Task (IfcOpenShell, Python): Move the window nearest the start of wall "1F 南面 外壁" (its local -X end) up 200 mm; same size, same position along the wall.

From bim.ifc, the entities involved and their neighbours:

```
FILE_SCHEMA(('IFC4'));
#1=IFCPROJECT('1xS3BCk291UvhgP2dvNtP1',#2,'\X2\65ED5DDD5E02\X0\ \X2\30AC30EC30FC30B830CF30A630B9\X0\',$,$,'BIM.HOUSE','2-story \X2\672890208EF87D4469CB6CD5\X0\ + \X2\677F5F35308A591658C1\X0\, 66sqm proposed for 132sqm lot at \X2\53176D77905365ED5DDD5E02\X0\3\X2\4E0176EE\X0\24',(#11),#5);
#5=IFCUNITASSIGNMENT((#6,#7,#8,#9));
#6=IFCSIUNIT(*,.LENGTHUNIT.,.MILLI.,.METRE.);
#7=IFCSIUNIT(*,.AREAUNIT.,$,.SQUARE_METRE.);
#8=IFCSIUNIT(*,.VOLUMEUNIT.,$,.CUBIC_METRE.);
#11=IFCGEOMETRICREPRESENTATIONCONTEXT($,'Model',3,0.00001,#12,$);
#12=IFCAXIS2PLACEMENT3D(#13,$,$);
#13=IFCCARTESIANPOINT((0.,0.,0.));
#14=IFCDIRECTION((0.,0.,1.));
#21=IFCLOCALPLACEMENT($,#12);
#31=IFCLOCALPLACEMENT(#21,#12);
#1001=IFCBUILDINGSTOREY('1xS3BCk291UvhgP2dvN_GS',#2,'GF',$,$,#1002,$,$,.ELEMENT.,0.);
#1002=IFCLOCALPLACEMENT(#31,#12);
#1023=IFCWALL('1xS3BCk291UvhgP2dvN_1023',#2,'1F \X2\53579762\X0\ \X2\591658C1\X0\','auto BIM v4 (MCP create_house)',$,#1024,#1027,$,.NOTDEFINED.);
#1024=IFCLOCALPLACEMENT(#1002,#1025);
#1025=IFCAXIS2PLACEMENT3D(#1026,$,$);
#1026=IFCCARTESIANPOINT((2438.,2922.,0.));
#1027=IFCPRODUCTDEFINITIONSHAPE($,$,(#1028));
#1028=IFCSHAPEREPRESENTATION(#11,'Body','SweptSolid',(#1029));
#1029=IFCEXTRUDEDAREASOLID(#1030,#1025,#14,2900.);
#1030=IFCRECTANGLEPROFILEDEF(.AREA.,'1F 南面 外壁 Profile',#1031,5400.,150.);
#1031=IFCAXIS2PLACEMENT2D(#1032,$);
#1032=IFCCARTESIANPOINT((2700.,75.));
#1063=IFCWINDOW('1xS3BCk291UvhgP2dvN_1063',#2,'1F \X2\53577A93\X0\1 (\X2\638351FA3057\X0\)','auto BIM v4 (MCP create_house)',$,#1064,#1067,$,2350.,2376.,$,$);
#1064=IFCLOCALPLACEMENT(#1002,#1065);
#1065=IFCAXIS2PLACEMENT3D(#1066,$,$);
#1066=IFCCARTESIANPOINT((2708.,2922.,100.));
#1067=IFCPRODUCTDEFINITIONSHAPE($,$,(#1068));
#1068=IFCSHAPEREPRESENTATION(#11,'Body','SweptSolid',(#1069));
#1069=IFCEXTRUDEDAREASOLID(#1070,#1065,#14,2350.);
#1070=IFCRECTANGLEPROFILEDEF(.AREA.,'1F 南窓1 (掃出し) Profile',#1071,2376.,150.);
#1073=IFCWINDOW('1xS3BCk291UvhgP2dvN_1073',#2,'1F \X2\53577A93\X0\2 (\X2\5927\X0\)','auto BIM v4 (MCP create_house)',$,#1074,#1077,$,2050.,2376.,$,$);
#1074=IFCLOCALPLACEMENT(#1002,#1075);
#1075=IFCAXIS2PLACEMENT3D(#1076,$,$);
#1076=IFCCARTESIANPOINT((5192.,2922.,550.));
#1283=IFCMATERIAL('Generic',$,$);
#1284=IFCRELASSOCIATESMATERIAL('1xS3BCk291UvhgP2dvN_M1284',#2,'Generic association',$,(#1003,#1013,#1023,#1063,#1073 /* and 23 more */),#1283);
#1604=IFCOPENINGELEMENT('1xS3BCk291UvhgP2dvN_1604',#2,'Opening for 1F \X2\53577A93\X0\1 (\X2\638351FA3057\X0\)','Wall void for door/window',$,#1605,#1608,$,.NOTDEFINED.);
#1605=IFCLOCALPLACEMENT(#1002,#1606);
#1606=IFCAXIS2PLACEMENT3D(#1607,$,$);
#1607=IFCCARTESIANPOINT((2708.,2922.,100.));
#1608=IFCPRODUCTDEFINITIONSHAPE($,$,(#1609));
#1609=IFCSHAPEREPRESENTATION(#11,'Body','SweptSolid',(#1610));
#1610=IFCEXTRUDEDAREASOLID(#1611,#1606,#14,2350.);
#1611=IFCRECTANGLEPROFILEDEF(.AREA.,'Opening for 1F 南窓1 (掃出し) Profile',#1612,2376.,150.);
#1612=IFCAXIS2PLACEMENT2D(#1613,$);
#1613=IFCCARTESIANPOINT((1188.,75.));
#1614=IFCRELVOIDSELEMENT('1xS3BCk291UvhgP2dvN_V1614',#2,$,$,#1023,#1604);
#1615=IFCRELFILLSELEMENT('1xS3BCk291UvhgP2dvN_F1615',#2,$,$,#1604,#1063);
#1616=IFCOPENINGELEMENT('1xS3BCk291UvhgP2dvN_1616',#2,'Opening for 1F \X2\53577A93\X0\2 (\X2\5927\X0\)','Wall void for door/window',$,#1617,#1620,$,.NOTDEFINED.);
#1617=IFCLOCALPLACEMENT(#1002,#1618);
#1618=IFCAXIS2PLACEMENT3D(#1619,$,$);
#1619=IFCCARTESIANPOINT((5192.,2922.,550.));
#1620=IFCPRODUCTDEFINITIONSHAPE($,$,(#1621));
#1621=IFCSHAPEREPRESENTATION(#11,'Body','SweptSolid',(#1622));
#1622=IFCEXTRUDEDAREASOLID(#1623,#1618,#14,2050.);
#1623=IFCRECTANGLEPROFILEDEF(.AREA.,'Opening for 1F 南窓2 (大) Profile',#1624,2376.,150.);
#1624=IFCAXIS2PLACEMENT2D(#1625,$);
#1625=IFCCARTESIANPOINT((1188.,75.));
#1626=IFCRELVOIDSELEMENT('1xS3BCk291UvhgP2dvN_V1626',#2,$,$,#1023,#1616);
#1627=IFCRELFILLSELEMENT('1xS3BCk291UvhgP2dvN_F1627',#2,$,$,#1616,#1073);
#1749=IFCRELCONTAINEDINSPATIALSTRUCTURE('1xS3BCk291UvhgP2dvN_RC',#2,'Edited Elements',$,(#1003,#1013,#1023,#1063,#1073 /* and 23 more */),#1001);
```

```python
import numpy as np
import ifcopenshell
import ifcopenshell.api.geometry
import ifcopenshell.util.placement
import ifcopenshell.util.unit

model = ifcopenshell.open("bim.ifc")
unit_scale = ifcopenshell.util.unit.calculate_unit_scale(model)

window = model.by_guid("1xS3BCk291UvhgP2dvN_1063")
opening = window.FillsVoids[0].RelatingOpeningElement
dz = 0.2 / unit_scale

shift = np.array([0.0, 0.0, dz])
# The window is not placed relative to its opening, so move both.
for product in (opening, window):
    matrix = ifcopenshell.util.placement.get_local_placement(product.ObjectPlacement)
    matrix[:3, 3] += shift
    ifcopenshell.api.geometry.edit_object_placement(model, product=product, matrix=matrix, is_si=False)

print(f"moved by {dz * unit_scale:+.3f} m")

model.write("bim-out.ifc")
```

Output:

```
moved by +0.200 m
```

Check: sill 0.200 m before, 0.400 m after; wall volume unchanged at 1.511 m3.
